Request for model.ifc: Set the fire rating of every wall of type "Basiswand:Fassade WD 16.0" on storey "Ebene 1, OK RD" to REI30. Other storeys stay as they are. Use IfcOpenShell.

First a look at what the model holds.

```python
import ifcopenshell
import ifcopenshell.util.element

model = ifcopenshell.open("model.ifc")
print(model.schema)
storey = next(s for s in model.by_type("IfcBuildingStorey") if s.Name == "Ebene 1, OK RD")
walls = [e for e in ifcopenshell.util.element.get_decomposition(storey) if e.is_a("IfcWall")]
seen = {}
for e in walls:
    element_type = ifcopenshell.util.element.get_type(e)
    key = (element_type.Name if element_type != e and element_type else None, ifcopenshell.util.element.get_pset(e, "Pset_WallCommon", "FireRating"))
    seen[key] = seen.get(key, 0) + 1
for (name, value), count in sorted(seen.items(), key=str):
    print(count, "x", name, "|", value)
```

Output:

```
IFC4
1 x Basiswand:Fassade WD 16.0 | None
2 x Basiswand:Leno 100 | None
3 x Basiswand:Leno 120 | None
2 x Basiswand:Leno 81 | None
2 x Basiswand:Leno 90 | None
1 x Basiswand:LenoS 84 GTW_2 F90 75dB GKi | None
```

```python
import ifcopenshell
import ifcopenshell.api.pset
import ifcopenshell.util.element

model = ifcopenshell.open("model.ifc")

storey = next(s for s in model.by_type("IfcBuildingStorey") if s.Name == "Ebene 1, OK RD")
walls = [e for e in ifcopenshell.util.element.get_decomposition(storey) if e.is_a("IfcWall")]

count = 0
for e in walls:
    element_type = ifcopenshell.util.element.get_type(e)
    if element_type in (None, e) or element_type.Name != "Basiswand:Fassade WD 16.0":
        continue
    # add_pset returns the element's existing set when there is one.
    pset = ifcopenshell.api.pset.add_pset(model, product=e, name="Pset_WallCommon")
    ifcopenshell.api.pset.edit_pset(model, pset=pset, properties={"FireRating": "REI30"})
    count += 1

print(count, "walls updated")

model.write("model_v2.ifc")
```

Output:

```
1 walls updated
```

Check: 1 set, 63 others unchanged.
